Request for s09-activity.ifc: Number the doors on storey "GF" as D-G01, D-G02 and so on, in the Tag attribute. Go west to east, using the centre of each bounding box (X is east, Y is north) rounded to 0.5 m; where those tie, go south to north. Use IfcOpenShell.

First a look at what the model holds.

```python
import ifcopenshell
import ifcopenshell.util.element
import ifcopenshell.util.placement

model = ifcopenshell.open("s09-activity.ifc")
print(model.schema)
storey = next(s for s in model.by_type("IfcBuildingStorey") if s.Name == "GF")
doors = [e for e in ifcopenshell.util.element.get_decomposition(storey) if e.is_a("IfcDoor")]
for e in sorted(doors, key=lambda e: e.id()):
    origin = ifcopenshell.util.placement.get_local_placement(e.ObjectPlacement)[:3, 3]
    print(e.id(), e.Tag, e.Name, origin.round(2) + 0.0, sep=" | ")
```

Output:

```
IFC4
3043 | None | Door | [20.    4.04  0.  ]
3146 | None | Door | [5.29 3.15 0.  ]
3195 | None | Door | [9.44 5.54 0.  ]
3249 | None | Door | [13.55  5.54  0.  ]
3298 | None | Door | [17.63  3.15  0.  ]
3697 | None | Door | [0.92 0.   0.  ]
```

```python
import ifcopenshell
import ifcopenshell.geom
import ifcopenshell.util.element
import ifcopenshell.util.shape

model = ifcopenshell.open("s09-activity.ifc")
settings = ifcopenshell.geom.settings()
settings.set("use-world-coords", True)


def centre(element):
    shape = ifcopenshell.geom.create_shape(settings, element)
    return ifcopenshell.util.shape.get_bbox_centroid(shape.geometry)


storey = next(s for s in model.by_type("IfcBuildingStorey") if s.Name == "GF")
doors = [e for e in ifcopenshell.util.element.get_decomposition(storey) if e.is_a("IfcDoor")]

# Insertion points can sit at a corner or the storey origin, so sort by the geometry (in metres).
centres = {e: centre(e) for e in doors}
doors.sort(key=lambda e: (round(centres[e][0] / 0.5), centres[e][1]))

for i, e in enumerate(doors, start=1):
    number = f"D-G{i:02d}"
    e.Tag = number
    print(e.id(), number)

model.write("s09-activity-out.ifc")
```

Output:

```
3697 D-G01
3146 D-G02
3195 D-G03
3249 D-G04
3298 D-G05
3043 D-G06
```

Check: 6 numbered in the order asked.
